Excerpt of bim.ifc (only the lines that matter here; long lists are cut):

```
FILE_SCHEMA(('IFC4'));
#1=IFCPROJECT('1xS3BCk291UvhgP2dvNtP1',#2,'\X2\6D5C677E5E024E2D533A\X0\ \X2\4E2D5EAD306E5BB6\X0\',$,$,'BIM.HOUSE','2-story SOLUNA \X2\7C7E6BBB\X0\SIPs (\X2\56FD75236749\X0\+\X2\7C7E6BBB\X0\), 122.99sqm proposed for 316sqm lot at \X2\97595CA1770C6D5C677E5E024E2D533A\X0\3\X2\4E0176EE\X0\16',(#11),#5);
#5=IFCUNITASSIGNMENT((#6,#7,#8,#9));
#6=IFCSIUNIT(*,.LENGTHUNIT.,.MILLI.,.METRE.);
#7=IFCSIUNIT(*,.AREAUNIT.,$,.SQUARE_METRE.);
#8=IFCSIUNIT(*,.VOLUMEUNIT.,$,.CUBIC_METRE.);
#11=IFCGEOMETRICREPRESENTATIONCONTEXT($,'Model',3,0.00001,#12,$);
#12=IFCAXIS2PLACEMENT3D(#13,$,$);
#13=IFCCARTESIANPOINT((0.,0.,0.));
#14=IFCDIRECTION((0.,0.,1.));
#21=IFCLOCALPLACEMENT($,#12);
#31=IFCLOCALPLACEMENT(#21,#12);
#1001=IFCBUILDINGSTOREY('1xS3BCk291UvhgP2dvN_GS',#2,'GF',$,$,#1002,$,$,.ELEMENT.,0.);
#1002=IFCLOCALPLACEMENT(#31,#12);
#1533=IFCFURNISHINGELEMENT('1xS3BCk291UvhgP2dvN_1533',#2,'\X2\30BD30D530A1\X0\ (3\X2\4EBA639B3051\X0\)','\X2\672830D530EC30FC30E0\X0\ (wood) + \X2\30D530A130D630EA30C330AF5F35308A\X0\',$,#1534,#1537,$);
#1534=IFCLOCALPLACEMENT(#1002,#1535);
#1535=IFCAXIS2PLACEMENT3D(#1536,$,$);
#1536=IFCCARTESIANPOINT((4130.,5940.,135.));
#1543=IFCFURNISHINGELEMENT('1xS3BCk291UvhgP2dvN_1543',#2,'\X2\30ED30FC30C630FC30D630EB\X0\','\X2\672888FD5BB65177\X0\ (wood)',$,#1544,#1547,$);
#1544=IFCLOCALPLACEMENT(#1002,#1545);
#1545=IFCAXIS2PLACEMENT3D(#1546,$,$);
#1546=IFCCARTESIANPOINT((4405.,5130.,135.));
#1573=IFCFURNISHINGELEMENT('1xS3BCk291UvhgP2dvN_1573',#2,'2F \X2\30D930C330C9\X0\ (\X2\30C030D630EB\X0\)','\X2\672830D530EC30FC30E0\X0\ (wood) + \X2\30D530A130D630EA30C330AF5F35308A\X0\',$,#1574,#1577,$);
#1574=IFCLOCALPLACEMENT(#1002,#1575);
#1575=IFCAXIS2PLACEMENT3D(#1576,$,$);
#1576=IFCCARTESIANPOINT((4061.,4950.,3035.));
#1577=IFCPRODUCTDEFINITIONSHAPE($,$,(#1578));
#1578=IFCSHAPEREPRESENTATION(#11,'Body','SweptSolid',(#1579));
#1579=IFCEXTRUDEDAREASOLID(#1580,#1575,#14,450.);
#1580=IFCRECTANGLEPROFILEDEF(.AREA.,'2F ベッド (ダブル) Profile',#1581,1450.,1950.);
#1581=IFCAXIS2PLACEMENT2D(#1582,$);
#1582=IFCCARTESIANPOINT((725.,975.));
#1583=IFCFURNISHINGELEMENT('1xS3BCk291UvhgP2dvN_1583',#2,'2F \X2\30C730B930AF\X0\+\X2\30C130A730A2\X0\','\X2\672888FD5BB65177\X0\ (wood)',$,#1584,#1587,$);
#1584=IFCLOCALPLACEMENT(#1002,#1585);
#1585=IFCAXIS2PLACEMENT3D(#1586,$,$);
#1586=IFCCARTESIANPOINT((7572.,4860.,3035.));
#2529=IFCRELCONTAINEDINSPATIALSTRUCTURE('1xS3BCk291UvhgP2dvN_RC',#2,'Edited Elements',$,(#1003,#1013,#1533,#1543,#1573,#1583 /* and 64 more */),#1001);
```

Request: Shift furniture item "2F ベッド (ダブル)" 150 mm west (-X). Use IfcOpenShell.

```python
import ifcopenshell
import ifcopenshell.api.geometry
import ifcopenshell.util.placement
import ifcopenshell.util.unit

model = ifcopenshell.open("bim.ifc")
unit_scale = ifcopenshell.util.unit.calculate_unit_scale(model)

item = model.by_id(1573)
matrix = ifcopenshell.util.placement.get_local_placement(item.ObjectPlacement)
matrix[0, 3] -= 0.15 / unit_scale
ifcopenshell.api.geometry.edit_object_placement(model, product=item, matrix=matrix, is_si=False)

print(ifcopenshell.util.placement.get_local_placement(item.ObjectPlacement).round(3) + 0.0)

model.write("bim_rev.ifc")
```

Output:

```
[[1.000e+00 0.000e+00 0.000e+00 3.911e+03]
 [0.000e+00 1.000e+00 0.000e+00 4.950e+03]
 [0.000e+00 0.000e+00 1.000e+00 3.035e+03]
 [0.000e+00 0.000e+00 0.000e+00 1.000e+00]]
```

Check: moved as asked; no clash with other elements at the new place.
